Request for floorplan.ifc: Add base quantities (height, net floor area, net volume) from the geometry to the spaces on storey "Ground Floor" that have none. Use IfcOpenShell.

First a look at what the model holds.

```python
import ifcopenshell
import ifcopenshell.util.element
import ifcopenshell.util.unit

model = ifcopenshell.open("floorplan.ifc")
print(model.schema)
for unit_type in ("LENGTHUNIT", "AREAUNIT", "VOLUMEUNIT"):
    print(unit_type, ifcopenshell.util.unit.calculate_unit_scale(model, unit_type))
storey = next(s for s in model.by_type("IfcBuildingStorey") if s.Name == "Ground Floor")
spaces = [e for e in ifcopenshell.util.element.get_decomposition(storey) if e.is_a("IfcSpace")]
for e in sorted(spaces, key=lambda e: e.id()):
    print(e.id(), e.is_a(), e.Name, list(ifcopenshell.util.element.get_psets(e, qtos_only=True)), sep=" | ")
```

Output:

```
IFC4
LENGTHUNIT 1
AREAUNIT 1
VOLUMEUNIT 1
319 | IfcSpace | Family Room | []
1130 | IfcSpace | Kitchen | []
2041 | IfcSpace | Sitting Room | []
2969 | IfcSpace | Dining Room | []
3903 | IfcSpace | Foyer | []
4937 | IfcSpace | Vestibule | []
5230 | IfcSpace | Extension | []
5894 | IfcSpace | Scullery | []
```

```python
import ifcopenshell
import ifcopenshell.api.pset
import ifcopenshell.geom
import ifcopenshell.util.element
import ifcopenshell.util.shape
import ifcopenshell.util.unit

model = ifcopenshell.open("floorplan.ifc")
unit_scale = ifcopenshell.util.unit.calculate_unit_scale(model)
area_scale = ifcopenshell.util.unit.calculate_unit_scale(model, "AREAUNIT")
volume_scale = ifcopenshell.util.unit.calculate_unit_scale(model, "VOLUMEUNIT")
settings = ifcopenshell.geom.settings()

storey = next(s for s in model.by_type("IfcBuildingStorey") if s.Name == "Ground Floor")
spaces = [e for e in ifcopenshell.util.element.get_decomposition(storey) if e.is_a("IfcSpace")]

for e in sorted(spaces, key=lambda e: e.id()):
    if ifcopenshell.util.element.get_psets(e, qtos_only=True, should_inherit=False):
        continue
    # Geometry comes back in metres, in the element's own axes.
    shape = ifcopenshell.geom.create_shape(settings, e)
    values = {
        "Height": ifcopenshell.util.shape.get_z(shape.geometry) / unit_scale,
        "NetFloorArea": ifcopenshell.util.shape.get_footprint_area(shape.geometry) / area_scale,
        "NetVolume": ifcopenshell.util.shape.get_volume(shape.geometry) / volume_scale,
    }
    qto = ifcopenshell.api.pset.add_qto(model, product=e, name="Qto_SpaceBaseQuantities")
    ifcopenshell.api.pset.edit_qto(model, qto=qto, properties=values)
    print(e.id(), {k: round(v, 3) for k, v in values.items()})

model.write("floorplan-out.ifc")
```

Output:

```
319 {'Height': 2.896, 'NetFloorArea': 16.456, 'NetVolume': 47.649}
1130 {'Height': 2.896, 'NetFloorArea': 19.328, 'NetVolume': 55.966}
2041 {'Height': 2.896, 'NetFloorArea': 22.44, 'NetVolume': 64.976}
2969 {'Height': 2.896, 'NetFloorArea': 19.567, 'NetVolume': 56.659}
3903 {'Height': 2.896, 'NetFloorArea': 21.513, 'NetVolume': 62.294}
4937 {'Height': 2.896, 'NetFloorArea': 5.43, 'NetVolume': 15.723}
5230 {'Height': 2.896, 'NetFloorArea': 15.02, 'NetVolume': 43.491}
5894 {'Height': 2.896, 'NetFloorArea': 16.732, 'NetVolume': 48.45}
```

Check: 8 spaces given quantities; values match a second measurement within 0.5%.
